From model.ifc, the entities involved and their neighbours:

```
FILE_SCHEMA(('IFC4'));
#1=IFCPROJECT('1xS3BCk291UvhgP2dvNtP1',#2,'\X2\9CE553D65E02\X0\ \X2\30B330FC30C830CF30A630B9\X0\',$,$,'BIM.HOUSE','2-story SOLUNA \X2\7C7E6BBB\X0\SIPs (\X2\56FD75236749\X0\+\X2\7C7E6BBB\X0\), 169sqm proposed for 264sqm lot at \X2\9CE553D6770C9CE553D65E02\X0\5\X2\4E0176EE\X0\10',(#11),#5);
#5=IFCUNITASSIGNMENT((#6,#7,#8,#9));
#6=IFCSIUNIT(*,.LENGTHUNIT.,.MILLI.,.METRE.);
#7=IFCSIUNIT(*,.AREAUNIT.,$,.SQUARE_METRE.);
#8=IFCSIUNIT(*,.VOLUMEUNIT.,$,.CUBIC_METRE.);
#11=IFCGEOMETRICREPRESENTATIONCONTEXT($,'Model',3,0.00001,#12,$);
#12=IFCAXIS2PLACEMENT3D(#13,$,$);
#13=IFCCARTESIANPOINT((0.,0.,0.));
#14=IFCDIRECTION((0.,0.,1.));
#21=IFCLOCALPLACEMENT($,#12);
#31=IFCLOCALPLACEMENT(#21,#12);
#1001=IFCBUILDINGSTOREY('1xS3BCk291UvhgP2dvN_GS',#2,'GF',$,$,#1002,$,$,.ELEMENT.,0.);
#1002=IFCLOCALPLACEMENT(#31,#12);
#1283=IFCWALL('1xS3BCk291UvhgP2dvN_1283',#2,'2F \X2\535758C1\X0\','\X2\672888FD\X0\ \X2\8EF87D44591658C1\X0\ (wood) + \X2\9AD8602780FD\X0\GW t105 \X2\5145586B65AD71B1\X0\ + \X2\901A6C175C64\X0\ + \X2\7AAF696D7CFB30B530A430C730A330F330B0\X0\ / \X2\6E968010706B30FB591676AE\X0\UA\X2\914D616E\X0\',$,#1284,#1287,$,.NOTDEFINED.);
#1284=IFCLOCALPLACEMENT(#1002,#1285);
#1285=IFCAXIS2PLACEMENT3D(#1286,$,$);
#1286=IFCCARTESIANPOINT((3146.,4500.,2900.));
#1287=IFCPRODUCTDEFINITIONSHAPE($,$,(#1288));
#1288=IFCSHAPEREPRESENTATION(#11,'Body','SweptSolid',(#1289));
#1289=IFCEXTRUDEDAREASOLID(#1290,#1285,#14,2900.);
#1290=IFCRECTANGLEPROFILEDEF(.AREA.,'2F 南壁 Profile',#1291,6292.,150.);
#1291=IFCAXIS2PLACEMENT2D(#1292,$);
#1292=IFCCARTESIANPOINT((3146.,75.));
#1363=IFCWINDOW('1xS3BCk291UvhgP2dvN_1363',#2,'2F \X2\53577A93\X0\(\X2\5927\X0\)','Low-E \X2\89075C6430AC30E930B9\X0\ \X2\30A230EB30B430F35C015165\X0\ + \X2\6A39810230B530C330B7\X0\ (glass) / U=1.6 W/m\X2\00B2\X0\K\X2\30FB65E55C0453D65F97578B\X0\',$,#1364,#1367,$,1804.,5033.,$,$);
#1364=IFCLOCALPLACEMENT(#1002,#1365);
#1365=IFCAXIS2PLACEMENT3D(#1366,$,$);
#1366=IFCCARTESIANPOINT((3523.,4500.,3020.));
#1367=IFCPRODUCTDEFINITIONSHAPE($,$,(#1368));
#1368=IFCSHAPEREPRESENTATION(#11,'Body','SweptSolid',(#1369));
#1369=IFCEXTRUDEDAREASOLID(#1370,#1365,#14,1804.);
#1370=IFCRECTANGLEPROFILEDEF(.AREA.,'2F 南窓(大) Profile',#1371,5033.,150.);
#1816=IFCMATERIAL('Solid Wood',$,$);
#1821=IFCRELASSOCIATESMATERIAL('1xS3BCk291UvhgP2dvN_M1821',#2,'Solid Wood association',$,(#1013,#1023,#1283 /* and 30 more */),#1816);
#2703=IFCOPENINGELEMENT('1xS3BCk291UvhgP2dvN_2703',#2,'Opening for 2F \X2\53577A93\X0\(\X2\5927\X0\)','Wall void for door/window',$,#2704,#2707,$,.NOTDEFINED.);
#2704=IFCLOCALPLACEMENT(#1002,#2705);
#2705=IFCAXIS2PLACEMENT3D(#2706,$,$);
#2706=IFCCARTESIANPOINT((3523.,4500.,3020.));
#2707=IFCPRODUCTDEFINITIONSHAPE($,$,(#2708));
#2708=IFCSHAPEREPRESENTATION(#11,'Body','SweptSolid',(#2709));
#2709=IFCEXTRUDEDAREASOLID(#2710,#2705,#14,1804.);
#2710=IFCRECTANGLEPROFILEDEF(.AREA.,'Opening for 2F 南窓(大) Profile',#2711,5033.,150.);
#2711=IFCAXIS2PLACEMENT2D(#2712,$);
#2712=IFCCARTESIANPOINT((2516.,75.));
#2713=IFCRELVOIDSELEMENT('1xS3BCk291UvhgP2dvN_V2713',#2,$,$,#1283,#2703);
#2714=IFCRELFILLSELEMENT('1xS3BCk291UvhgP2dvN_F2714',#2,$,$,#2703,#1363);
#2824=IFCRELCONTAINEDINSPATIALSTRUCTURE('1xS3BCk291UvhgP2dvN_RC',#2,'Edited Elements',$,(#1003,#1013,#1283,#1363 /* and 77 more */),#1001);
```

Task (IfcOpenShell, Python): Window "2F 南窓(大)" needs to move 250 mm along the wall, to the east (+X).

```python
import ifcopenshell
import ifcopenshell.api.geometry
import ifcopenshell.util.placement

model = ifcopenshell.open("model.ifc")

window = model.by_guid("1xS3BCk291UvhgP2dvN_1363")
opening = window.FillsVoids[0].RelatingOpeningElement
wall = opening.VoidsElements[0].RelatingBuildingElement

wall_matrix = ifcopenshell.util.placement.get_local_placement(wall.ObjectPlacement)
shift = wall_matrix[:3, 0] * 250.0
before = ifcopenshell.util.placement.get_local_placement(window.ObjectPlacement)[:3, 3].copy()

# The window is not placed relative to its opening, so move both.
for product in (opening, window):
    matrix = ifcopenshell.util.placement.get_local_placement(product.ObjectPlacement)
    matrix[:3, 3] += shift
    ifcopenshell.api.geometry.edit_object_placement(model, product=product, matrix=matrix, is_si=False)

after = ifcopenshell.util.placement.get_local_placement(window.ObjectPlacement)[:3, 3]
print("window moved by", (after - before).round(3) + 0.0)

model.write("model-out.ifc")
```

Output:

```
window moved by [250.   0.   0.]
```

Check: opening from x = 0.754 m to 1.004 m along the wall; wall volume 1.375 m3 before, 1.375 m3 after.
